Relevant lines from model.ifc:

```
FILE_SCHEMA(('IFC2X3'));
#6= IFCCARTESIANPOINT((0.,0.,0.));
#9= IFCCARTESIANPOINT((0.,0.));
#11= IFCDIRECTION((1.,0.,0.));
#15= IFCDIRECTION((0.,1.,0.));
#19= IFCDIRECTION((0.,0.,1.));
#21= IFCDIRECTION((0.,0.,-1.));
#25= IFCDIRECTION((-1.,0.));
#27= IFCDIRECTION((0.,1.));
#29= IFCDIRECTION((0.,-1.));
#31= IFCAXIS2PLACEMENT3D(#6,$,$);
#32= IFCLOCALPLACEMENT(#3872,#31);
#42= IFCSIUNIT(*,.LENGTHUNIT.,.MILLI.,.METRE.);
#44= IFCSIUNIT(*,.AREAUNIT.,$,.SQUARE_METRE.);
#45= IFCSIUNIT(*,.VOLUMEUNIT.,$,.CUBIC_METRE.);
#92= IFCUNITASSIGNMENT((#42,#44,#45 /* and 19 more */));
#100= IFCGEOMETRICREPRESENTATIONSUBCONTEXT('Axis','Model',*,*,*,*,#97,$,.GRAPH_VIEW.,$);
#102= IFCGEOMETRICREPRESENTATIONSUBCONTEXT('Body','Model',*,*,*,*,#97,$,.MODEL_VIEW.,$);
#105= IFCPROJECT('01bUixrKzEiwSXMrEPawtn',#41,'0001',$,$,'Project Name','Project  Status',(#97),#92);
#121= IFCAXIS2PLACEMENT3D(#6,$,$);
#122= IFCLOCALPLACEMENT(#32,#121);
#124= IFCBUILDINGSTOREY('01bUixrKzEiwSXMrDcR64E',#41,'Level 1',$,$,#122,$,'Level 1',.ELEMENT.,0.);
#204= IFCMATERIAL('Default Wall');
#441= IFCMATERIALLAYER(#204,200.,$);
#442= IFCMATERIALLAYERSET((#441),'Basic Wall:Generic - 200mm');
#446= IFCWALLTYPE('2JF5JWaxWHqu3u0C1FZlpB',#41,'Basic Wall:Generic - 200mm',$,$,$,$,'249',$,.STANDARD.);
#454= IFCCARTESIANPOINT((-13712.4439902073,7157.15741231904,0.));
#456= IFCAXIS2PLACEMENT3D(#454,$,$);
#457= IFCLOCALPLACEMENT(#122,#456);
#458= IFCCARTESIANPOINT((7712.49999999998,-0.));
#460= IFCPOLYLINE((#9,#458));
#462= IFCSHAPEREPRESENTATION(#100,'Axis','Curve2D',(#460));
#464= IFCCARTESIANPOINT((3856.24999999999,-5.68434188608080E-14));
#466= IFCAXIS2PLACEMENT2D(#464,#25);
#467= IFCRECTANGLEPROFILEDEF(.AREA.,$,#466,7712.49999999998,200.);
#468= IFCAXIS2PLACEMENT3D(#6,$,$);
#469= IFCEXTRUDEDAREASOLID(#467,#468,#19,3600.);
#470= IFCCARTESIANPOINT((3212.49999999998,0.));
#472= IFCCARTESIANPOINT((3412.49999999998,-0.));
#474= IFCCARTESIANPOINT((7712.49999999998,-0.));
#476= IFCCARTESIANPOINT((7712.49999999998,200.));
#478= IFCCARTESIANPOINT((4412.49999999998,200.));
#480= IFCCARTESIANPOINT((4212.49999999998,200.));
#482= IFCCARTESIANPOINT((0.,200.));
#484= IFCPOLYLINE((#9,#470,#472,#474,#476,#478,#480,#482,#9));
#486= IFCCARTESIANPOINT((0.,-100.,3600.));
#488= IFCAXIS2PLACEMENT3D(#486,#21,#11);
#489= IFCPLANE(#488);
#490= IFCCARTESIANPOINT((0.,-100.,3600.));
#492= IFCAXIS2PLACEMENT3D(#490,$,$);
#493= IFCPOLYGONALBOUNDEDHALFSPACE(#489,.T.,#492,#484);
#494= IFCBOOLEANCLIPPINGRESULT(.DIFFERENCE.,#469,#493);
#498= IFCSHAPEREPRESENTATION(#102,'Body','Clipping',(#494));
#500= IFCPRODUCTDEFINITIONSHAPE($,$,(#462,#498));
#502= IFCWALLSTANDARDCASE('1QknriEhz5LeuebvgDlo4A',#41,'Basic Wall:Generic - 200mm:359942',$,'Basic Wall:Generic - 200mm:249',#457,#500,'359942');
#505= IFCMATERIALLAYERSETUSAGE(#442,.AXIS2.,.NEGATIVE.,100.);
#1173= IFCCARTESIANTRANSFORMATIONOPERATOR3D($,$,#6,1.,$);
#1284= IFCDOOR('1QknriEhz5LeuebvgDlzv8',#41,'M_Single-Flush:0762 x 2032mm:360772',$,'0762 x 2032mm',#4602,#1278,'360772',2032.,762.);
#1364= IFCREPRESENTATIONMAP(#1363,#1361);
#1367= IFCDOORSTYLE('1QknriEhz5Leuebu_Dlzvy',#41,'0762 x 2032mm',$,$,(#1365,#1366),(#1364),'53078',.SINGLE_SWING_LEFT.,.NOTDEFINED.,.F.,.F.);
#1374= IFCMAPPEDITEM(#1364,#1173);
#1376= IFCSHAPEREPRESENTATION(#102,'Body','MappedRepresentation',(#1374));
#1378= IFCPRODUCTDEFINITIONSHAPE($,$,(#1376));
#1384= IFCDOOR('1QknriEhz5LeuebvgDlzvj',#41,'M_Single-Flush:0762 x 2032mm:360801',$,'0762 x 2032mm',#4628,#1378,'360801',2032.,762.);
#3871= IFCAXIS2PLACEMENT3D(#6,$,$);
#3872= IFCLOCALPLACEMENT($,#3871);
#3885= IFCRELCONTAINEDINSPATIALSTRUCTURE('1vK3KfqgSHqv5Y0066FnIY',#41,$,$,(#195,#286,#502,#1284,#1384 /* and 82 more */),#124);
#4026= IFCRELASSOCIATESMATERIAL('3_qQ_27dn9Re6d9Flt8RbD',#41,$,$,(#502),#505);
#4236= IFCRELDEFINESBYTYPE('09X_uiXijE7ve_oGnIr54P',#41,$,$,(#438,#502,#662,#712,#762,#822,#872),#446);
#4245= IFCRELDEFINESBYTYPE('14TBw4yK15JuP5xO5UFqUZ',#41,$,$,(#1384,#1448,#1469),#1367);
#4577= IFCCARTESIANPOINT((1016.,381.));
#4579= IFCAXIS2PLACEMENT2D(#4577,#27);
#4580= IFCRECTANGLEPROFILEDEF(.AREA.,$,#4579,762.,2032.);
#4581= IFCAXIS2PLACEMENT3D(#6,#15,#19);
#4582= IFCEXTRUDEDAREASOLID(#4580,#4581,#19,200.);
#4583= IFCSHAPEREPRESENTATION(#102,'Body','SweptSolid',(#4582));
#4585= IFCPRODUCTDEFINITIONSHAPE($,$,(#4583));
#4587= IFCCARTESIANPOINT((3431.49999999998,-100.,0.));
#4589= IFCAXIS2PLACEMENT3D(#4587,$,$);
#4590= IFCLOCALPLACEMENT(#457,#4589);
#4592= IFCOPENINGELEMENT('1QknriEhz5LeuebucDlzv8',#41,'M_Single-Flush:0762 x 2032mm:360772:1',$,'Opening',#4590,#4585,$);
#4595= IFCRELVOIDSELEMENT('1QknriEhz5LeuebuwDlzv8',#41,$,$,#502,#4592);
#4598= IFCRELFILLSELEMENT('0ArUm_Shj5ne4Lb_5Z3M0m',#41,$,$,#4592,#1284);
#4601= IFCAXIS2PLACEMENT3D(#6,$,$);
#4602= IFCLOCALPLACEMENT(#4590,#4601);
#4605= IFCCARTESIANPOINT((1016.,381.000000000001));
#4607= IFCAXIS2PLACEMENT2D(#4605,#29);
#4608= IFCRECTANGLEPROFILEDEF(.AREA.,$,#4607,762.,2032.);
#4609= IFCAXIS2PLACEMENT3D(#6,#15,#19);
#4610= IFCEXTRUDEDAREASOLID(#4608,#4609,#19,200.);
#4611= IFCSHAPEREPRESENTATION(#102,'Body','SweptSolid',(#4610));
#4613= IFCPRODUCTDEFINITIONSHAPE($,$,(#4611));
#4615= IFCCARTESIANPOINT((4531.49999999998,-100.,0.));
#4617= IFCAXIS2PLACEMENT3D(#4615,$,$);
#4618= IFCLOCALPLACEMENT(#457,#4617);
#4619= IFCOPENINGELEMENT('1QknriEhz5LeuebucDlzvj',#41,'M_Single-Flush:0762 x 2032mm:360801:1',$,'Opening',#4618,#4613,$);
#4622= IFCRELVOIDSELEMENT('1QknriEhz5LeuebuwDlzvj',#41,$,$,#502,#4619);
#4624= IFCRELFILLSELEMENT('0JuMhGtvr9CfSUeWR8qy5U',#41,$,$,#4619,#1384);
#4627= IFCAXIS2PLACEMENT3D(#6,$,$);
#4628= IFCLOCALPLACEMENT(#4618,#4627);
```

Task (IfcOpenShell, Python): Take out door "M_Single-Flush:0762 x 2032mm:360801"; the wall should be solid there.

```python
import ifcopenshell
import ifcopenshell.api.feature
import ifcopenshell.api.root
import ifcopenshell.geom
import ifcopenshell.util.shape

model = ifcopenshell.open("model.ifc")
settings = ifcopenshell.geom.settings()


def volume(element):
    """Net volume in cubic metres, openings subtracted."""
    shape = ifcopenshell.geom.create_shape(settings, element)
    return ifcopenshell.util.shape.get_volume(shape.geometry)


door = model.by_guid("1QknriEhz5LeuebvgDlzvj")
opening = door.FillsVoids[0].RelatingOpeningElement
wall = opening.VoidsElements[0].RelatingBuildingElement
before = volume(wall)

ifcopenshell.api.root.remove_product(model, product=door)
ifcopenshell.api.feature.remove_feature(model, feature=opening)

after = volume(wall)

print(f"wall volume {before:.3f} -> {after:.3f} m3")

model.write("model_edited.ifc")
```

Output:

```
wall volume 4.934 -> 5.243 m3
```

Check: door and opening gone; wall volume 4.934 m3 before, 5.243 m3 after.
